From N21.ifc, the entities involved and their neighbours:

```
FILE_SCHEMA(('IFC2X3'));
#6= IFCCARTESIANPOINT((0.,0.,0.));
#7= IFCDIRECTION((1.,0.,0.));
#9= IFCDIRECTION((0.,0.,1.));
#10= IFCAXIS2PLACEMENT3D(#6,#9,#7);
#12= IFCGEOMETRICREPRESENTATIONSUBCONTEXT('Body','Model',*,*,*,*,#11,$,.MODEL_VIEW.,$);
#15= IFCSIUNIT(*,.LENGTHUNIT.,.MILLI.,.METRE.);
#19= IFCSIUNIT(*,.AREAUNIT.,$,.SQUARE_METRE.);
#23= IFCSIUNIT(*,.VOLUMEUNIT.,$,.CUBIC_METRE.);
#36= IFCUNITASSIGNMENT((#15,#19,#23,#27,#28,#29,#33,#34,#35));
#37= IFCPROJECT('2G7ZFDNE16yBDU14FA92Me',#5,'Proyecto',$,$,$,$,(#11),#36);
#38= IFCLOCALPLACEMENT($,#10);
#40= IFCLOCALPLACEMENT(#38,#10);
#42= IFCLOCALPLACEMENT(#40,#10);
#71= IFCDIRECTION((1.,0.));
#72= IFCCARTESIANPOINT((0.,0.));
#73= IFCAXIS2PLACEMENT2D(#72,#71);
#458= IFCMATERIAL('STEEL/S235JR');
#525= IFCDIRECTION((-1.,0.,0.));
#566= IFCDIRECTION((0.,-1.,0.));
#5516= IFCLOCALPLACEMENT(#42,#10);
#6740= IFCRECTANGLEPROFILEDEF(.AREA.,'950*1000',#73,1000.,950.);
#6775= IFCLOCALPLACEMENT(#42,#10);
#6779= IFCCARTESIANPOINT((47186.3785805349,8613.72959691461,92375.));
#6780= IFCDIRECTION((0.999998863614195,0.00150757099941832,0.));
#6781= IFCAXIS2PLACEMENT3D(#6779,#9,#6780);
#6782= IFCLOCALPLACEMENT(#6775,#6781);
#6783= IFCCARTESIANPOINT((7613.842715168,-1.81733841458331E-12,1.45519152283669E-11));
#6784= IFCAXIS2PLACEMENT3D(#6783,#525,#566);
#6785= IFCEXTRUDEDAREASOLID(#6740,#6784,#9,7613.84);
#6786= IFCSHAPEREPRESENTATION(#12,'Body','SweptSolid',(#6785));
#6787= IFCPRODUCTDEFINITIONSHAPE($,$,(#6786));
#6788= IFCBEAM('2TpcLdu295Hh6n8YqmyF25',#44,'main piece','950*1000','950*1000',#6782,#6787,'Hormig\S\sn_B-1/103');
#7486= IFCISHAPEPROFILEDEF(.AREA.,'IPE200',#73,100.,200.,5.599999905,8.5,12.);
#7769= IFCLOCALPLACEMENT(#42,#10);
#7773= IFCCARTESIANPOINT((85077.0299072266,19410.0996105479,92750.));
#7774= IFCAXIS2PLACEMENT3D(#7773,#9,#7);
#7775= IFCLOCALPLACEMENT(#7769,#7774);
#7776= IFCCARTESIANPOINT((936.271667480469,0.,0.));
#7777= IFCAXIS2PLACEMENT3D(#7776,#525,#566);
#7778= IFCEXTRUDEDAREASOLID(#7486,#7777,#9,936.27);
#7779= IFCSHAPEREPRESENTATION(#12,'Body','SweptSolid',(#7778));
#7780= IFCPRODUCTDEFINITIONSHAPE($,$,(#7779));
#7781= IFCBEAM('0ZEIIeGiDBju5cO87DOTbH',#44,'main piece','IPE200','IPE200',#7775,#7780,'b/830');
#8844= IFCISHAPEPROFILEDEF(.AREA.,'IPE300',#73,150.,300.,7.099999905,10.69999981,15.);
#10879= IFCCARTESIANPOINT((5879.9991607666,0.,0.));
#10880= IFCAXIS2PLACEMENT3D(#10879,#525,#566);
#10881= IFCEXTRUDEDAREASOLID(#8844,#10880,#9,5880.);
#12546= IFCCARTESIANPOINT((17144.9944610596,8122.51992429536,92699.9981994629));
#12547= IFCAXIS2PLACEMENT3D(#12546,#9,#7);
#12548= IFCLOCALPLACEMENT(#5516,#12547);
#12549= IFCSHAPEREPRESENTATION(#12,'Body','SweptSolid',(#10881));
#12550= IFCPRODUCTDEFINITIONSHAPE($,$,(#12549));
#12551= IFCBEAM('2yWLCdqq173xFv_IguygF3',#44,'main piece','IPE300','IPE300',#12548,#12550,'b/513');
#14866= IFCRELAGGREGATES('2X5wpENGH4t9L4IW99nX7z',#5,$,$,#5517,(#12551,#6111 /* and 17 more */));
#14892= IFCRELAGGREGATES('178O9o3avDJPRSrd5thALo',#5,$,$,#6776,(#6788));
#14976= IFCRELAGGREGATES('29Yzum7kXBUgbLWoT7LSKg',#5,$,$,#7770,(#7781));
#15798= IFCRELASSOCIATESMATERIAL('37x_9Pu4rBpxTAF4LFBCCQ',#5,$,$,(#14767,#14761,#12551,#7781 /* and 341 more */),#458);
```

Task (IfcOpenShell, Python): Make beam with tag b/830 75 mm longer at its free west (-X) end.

```python
import ifcopenshell
import ifcopenshell.util.representation
import ifcopenshell.util.unit

model = ifcopenshell.open("N21.ifc")
unit_scale = ifcopenshell.util.unit.calculate_unit_scale(model)

member = model.by_guid("0ZEIIeGiDBju5cO87DOTbH")
change = 0.075 / unit_scale

# The extrusion runs towards the end named, so only its depth changes.
body = ifcopenshell.util.representation.get_representation(member, "Model", "Body")
solid = body.Items[0]
old_length = solid.Depth
solid.Depth += change

print(f"length {old_length:g} -> {solid.Depth:g}")

model.write("N21_updated.ifc")
```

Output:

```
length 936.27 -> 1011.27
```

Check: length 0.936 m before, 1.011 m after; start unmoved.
